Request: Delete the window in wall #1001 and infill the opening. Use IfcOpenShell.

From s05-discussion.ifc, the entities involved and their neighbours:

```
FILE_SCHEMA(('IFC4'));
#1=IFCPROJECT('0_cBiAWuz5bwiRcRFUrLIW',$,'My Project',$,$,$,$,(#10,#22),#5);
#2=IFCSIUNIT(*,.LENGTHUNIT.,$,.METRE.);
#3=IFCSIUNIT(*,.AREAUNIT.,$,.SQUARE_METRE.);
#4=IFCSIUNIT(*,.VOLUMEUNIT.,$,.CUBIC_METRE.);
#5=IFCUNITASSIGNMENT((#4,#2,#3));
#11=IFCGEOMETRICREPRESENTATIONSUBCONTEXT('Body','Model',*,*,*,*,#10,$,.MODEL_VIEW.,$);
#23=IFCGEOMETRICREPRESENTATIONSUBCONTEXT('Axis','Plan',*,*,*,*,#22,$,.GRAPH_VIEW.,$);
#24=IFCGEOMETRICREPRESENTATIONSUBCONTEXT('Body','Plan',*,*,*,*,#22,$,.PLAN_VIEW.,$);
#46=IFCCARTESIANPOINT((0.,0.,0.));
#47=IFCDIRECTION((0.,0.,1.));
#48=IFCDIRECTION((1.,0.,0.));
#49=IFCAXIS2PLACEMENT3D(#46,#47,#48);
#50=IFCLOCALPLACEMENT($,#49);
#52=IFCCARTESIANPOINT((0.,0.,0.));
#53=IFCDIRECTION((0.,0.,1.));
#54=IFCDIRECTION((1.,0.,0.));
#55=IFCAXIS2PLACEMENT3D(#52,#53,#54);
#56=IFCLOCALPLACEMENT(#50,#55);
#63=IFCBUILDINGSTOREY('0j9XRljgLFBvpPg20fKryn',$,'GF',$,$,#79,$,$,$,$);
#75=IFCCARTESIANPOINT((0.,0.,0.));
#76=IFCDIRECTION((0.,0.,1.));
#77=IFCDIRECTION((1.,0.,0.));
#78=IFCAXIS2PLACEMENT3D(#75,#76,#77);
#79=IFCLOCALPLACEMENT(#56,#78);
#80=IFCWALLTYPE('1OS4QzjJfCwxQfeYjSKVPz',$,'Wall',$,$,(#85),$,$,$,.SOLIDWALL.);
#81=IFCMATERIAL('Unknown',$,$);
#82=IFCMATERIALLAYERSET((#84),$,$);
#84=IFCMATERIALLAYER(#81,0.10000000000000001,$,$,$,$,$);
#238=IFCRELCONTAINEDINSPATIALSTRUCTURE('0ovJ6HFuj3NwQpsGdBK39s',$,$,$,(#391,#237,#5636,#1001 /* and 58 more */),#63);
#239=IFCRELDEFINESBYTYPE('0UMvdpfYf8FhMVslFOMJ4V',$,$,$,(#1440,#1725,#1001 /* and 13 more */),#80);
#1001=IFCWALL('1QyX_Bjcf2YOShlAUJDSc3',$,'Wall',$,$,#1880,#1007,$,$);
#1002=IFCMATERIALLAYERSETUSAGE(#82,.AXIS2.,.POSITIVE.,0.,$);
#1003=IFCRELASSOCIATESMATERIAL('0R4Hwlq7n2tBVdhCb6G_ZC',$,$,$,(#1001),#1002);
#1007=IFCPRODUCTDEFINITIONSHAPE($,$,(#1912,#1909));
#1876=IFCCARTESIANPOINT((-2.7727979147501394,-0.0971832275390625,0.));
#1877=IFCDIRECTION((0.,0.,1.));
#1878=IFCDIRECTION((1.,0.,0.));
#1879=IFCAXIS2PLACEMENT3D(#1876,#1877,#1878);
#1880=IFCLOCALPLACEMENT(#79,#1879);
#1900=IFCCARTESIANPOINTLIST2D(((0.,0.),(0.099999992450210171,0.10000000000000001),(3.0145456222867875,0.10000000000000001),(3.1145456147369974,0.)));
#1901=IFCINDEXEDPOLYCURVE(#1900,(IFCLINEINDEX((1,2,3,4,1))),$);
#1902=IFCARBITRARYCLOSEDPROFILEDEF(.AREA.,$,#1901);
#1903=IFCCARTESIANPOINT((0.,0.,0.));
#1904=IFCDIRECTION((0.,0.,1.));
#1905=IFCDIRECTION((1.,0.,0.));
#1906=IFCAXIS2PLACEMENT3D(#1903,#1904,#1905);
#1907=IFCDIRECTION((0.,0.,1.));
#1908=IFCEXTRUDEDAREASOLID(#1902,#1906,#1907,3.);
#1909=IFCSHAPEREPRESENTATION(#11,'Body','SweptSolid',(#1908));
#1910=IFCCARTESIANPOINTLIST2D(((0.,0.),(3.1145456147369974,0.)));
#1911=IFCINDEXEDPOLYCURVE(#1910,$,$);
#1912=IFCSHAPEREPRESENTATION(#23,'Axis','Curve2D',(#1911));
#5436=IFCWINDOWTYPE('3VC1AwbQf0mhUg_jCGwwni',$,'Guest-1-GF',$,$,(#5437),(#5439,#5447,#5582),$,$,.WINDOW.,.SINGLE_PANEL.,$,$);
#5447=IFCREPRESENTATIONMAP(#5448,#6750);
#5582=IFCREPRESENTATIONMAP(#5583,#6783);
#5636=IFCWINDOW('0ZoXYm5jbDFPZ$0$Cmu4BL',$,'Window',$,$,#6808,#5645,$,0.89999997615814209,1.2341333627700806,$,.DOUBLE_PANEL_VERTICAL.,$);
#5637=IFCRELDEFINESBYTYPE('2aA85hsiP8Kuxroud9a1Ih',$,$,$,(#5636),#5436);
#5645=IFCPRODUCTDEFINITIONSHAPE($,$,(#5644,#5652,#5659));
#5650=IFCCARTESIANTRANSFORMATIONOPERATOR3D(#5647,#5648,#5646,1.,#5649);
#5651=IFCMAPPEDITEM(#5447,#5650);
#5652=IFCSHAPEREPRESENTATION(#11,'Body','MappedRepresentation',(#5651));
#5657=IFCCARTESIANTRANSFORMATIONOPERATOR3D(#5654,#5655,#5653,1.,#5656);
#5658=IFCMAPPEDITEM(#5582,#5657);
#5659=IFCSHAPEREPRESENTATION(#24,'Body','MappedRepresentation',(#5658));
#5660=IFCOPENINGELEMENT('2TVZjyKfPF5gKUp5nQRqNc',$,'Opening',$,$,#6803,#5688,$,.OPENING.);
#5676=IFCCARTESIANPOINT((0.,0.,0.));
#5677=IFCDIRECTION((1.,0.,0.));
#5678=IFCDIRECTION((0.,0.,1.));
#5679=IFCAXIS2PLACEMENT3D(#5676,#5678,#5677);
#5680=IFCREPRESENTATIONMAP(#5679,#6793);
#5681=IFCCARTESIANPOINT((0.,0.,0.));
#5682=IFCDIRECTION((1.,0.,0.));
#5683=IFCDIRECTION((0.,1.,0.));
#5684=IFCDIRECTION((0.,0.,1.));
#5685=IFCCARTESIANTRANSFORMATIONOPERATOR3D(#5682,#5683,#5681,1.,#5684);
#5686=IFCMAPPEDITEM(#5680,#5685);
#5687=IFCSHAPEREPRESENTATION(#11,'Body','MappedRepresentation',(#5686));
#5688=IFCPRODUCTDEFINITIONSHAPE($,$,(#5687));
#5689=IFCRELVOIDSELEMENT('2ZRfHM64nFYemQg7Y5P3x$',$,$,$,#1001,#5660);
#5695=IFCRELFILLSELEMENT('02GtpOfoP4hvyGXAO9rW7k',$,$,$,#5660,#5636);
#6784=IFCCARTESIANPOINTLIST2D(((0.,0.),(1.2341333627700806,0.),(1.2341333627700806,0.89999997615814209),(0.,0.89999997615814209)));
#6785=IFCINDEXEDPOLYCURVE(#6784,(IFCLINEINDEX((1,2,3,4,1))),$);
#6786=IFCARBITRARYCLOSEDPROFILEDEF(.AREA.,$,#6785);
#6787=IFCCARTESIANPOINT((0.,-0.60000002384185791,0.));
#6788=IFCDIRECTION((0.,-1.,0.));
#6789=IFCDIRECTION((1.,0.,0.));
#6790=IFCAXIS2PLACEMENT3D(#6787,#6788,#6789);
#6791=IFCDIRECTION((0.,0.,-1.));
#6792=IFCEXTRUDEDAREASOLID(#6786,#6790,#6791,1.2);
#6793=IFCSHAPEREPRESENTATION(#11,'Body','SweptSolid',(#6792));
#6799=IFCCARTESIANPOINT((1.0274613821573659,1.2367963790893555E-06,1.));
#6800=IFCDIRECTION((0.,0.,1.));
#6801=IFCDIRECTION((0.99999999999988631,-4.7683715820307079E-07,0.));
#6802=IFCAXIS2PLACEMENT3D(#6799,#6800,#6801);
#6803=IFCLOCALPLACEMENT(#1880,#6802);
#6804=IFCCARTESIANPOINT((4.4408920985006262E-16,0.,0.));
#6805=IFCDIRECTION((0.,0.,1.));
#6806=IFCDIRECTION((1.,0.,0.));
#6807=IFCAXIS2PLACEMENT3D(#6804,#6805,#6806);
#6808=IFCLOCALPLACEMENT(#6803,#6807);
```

```python
import ifcopenshell
import ifcopenshell.api.feature
import ifcopenshell.api.root
import ifcopenshell.geom
import ifcopenshell.util.shape

model = ifcopenshell.open("s05-discussion.ifc")
settings = ifcopenshell.geom.settings()


def volume(element):
    """Net volume in cubic metres, openings subtracted."""
    shape = ifcopenshell.geom.create_shape(settings, element)
    return ifcopenshell.util.shape.get_volume(shape.geometry)


window = model.by_guid("0ZoXYm5jbDFPZ$0$Cmu4BL")
opening = window.FillsVoids[0].RelatingOpeningElement
wall = opening.VoidsElements[0].RelatingBuildingElement
before = volume(wall)

ifcopenshell.api.root.remove_product(model, product=window)
ifcopenshell.api.feature.remove_feature(model, feature=opening)

after = volume(wall)

print(f"wall volume {before:.3f} -> {after:.3f} m3")

model.write("s05-discussion_rev.ifc")
```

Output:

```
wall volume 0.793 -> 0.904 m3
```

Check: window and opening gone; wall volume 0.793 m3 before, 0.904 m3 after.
